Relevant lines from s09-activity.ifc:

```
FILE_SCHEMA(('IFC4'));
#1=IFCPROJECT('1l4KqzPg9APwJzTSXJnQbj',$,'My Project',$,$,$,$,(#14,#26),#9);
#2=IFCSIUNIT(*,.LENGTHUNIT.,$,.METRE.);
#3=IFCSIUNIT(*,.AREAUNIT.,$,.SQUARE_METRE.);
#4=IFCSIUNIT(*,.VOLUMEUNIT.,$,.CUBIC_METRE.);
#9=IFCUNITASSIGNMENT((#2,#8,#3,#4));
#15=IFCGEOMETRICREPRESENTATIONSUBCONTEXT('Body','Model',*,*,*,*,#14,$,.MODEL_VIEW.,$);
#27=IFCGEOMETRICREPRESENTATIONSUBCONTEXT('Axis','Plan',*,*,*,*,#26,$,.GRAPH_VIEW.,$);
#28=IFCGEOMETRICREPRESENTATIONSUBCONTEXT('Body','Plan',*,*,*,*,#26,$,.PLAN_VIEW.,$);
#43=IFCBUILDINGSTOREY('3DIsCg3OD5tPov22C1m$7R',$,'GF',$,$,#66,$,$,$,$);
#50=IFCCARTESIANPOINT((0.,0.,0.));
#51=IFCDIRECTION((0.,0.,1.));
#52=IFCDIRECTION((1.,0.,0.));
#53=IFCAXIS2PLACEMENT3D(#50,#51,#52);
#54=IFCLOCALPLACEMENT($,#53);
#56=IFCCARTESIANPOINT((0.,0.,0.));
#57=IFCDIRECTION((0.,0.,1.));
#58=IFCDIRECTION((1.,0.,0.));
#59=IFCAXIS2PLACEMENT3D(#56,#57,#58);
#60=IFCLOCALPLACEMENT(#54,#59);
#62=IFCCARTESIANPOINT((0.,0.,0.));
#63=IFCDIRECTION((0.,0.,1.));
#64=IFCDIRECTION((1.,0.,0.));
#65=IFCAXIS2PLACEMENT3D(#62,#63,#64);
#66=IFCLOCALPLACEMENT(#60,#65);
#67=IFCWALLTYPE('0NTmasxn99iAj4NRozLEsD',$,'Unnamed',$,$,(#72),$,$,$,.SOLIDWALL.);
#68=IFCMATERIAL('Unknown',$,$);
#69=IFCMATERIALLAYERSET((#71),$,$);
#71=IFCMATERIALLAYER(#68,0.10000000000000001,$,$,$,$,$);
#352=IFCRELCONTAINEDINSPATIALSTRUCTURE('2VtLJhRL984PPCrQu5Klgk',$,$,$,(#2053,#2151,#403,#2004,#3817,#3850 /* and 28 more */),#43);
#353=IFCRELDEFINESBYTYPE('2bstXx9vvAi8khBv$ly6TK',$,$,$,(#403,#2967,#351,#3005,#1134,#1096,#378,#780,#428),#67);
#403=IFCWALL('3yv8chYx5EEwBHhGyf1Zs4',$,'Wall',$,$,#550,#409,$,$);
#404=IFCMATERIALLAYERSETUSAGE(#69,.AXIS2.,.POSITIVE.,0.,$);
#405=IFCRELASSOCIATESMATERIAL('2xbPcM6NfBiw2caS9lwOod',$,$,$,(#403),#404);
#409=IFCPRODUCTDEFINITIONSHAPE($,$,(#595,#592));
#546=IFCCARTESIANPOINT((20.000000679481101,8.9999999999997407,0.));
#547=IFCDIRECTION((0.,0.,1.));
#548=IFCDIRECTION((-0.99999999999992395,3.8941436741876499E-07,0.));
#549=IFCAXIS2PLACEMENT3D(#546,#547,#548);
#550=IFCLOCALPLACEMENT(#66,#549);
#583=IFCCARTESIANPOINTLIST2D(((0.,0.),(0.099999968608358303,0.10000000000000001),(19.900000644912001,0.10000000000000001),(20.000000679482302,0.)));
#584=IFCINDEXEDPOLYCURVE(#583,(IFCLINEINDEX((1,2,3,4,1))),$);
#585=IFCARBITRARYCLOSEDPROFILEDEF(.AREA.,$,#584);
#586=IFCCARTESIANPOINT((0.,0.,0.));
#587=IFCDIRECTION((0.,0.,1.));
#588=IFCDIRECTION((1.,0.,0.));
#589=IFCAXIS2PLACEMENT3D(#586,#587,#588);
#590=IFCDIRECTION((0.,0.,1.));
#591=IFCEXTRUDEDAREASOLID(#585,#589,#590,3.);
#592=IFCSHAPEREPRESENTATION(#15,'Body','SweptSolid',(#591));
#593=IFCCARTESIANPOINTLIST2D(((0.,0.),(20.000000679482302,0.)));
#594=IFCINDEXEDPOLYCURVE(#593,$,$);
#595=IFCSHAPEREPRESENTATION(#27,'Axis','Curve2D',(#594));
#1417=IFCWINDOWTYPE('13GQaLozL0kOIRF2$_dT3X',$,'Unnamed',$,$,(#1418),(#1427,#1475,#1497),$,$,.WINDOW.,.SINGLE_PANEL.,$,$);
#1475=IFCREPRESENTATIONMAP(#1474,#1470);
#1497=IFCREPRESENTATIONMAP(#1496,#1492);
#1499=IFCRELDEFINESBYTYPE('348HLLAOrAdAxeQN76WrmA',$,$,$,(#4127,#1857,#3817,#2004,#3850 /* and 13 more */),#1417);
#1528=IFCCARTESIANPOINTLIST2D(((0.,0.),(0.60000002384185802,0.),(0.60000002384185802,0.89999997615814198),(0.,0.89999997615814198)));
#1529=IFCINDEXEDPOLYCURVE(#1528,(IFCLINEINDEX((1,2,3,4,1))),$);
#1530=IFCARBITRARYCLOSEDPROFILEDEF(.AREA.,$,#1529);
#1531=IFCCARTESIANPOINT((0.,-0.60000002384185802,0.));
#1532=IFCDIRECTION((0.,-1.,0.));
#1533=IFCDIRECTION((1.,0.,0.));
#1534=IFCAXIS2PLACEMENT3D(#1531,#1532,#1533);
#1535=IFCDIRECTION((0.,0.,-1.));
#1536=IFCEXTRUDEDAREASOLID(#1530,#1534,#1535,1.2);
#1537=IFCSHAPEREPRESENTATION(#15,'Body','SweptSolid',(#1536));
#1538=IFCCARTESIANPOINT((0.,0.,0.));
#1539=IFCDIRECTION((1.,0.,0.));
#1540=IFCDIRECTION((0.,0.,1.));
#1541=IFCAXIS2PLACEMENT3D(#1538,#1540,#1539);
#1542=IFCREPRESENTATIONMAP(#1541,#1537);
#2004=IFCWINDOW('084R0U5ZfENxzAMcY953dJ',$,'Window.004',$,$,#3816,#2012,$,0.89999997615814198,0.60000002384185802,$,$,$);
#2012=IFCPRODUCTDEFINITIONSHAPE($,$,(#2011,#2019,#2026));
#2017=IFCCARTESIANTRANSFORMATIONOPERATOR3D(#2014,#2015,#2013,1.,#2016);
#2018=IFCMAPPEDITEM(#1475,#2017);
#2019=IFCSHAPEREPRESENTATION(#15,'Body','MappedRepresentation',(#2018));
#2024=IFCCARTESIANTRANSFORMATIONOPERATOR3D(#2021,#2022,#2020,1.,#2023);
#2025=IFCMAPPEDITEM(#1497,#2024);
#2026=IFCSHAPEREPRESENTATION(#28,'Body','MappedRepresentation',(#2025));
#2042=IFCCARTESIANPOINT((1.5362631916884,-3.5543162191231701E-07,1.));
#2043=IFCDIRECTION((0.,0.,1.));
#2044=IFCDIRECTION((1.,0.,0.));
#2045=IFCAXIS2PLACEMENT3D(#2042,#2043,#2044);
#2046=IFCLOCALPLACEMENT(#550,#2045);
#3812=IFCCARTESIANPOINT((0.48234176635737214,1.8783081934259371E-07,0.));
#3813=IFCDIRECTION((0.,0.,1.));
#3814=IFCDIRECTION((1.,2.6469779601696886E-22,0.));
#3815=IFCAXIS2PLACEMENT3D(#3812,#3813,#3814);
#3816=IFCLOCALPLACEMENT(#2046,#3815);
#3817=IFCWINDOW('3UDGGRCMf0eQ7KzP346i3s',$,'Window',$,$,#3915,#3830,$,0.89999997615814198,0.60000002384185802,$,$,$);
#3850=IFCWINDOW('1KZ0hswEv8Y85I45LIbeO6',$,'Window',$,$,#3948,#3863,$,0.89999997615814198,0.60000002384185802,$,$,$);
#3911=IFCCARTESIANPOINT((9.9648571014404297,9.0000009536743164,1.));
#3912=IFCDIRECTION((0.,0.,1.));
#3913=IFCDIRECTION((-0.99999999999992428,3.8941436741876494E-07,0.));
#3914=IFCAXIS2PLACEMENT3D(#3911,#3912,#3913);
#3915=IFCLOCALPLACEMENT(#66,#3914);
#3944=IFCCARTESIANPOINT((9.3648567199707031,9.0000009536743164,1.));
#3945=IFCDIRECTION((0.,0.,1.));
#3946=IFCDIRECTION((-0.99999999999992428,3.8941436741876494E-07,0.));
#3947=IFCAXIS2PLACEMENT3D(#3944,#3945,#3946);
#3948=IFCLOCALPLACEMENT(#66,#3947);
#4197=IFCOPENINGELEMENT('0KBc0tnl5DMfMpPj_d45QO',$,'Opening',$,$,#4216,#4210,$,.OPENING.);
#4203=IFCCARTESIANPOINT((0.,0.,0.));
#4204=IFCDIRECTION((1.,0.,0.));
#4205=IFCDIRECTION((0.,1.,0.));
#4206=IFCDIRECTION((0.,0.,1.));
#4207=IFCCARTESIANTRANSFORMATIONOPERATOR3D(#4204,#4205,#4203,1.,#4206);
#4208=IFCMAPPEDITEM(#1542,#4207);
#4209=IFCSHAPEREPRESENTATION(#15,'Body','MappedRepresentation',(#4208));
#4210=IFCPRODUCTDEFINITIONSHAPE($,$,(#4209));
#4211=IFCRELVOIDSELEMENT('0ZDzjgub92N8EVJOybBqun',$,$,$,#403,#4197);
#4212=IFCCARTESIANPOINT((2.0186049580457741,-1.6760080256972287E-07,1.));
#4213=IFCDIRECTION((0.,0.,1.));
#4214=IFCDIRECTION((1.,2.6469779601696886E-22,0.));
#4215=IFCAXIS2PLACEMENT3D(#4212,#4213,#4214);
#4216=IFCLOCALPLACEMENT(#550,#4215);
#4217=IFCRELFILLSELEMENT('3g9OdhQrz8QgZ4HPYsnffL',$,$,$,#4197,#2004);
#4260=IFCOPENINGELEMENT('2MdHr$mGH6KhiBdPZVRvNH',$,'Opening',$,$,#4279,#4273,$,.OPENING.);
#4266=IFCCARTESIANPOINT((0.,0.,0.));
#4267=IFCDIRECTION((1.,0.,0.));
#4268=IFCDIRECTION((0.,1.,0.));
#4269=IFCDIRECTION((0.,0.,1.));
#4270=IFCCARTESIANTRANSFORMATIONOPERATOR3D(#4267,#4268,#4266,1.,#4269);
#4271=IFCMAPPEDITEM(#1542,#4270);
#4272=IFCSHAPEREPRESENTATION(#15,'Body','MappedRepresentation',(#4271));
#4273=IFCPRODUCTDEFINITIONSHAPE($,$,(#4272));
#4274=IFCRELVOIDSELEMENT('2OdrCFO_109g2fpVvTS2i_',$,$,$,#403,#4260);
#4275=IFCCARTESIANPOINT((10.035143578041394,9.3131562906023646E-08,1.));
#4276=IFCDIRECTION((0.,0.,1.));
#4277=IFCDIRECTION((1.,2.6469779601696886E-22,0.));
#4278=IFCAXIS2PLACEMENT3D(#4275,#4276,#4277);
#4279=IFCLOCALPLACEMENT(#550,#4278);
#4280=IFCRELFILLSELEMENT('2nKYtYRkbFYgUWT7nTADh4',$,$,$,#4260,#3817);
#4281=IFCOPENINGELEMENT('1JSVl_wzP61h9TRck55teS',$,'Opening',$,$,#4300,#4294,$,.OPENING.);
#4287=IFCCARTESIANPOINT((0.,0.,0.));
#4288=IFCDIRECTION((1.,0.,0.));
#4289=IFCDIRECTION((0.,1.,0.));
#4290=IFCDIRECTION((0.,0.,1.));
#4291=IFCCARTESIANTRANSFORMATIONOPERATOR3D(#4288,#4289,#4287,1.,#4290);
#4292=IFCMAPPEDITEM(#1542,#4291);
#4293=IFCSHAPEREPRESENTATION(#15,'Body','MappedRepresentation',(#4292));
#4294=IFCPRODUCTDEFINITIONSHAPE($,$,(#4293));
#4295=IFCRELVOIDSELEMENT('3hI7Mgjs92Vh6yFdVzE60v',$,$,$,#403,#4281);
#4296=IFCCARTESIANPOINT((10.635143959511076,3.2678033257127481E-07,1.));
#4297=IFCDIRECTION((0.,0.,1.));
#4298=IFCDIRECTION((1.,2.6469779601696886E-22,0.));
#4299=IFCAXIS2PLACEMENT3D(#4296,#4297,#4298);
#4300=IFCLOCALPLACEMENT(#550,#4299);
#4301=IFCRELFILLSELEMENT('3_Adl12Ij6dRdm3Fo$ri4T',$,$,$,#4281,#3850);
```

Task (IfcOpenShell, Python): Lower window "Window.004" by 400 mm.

```python
import numpy as np
import ifcopenshell
import ifcopenshell.api.geometry
import ifcopenshell.util.placement
import ifcopenshell.util.unit

model = ifcopenshell.open("s09-activity.ifc")
unit_scale = ifcopenshell.util.unit.calculate_unit_scale(model)

window = model.by_guid("084R0U5ZfENxzAMcY953dJ")
opening = window.FillsVoids[0].RelatingOpeningElement
dz = -0.4 / unit_scale

shift = np.array([0.0, 0.0, dz])
# The window is not placed relative to its opening, so move both.
for product in (opening, window):
    matrix = ifcopenshell.util.placement.get_local_placement(product.ObjectPlacement)
    matrix[:3, 3] += shift
    ifcopenshell.api.geometry.edit_object_placement(model, product=product, matrix=matrix, is_si=False)

print(f"moved by {dz * unit_scale:+.3f} m")

model.write("s09-activity_v2.ifc")
```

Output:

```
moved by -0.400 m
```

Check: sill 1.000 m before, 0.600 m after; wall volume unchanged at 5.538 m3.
